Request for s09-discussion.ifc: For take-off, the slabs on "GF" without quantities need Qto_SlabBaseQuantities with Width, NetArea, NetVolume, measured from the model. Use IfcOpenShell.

First a look at what the model holds.

```python
import ifcopenshell
import ifcopenshell.util.element
import ifcopenshell.util.unit

model = ifcopenshell.open("s09-discussion.ifc")
print(model.schema)
for unit_type in ("LENGTHUNIT", "AREAUNIT", "VOLUMEUNIT"):
    print(unit_type, ifcopenshell.util.unit.calculate_unit_scale(model, unit_type))
storey = next(s for s in model.by_type("IfcBuildingStorey") if s.Name == "GF")
slabs = [e for e in ifcopenshell.util.element.get_decomposition(storey) if e.is_a("IfcSlab")]
for e in sorted(slabs, key=lambda e: e.id()):
    print(e.id(), e.is_a(), e.Name, list(ifcopenshell.util.element.get_psets(e, qtos_only=True)), sep=" | ")
```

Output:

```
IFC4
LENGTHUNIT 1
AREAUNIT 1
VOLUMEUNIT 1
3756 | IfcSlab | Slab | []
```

```python
import ifcopenshell
import ifcopenshell.api.pset
import ifcopenshell.geom
import ifcopenshell.util.element
import ifcopenshell.util.shape
import ifcopenshell.util.unit

model = ifcopenshell.open("s09-discussion.ifc")
unit_scale = ifcopenshell.util.unit.calculate_unit_scale(model)
area_scale = ifcopenshell.util.unit.calculate_unit_scale(model, "AREAUNIT")
volume_scale = ifcopenshell.util.unit.calculate_unit_scale(model, "VOLUMEUNIT")
settings = ifcopenshell.geom.settings()

storey = next(s for s in model.by_type("IfcBuildingStorey") if s.Name == "GF")
slabs = [e for e in ifcopenshell.util.element.get_decomposition(storey) if e.is_a("IfcSlab")]

for e in sorted(slabs, key=lambda e: e.id()):
    if ifcopenshell.util.element.get_psets(e, qtos_only=True, should_inherit=False):
        continue
    # Geometry comes back in metres, in the element's own axes.
    shape = ifcopenshell.geom.create_shape(settings, e)
    values = {
        "Width": ifcopenshell.util.shape.get_z(shape.geometry) / unit_scale,
        "NetArea": ifcopenshell.util.shape.get_footprint_area(shape.geometry) / area_scale,
        "NetVolume": ifcopenshell.util.shape.get_volume(shape.geometry) / volume_scale,
    }
    qto = ifcopenshell.api.pset.add_qto(model, product=e, name="Qto_SlabBaseQuantities")
    ifcopenshell.api.pset.edit_qto(model, qto=qto, properties=values)
    print(e.id(), {k: round(v, 3) for k, v in values.items()})

model.write("s09-discussion_updated.ifc")
```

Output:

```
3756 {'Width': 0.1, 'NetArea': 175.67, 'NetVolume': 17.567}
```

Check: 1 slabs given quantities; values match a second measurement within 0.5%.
